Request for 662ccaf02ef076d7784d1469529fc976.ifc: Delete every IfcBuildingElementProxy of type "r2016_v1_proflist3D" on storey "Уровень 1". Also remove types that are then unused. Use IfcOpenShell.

First a look at what the model holds.

```python
import ifcopenshell
import ifcopenshell.util.element

model = ifcopenshell.open("662ccaf02ef076d7784d1469529fc976.ifc")
print(model.schema)
storey = next(s for s in model.by_type("IfcBuildingStorey") if s.Name == "Уровень 1")
proxies = [e for e in ifcopenshell.util.element.get_decomposition(storey) if e.is_a("IfcBuildingElementProxy")]
seen = {}
for e in proxies:
    element_type = ifcopenshell.util.element.get_type(e)
    name = element_type.Name if element_type not in (None, e) else None
    seen[name] = seen.get(name, 0) + 1
for name, count in sorted(seen.items(), key=str):
    print(count, "x", name)
```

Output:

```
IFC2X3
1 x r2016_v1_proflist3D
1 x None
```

```python
import ifcopenshell
import ifcopenshell.api.root
import ifcopenshell.util.element

model = ifcopenshell.open("662ccaf02ef076d7784d1469529fc976.ifc")

storey = next(s for s in model.by_type("IfcBuildingStorey") if s.Name == "Уровень 1")
proxies = [e for e in ifcopenshell.util.element.get_decomposition(storey) if e.is_a("IfcBuildingElementProxy")]
targets = [e for e in proxies if (t := ifcopenshell.util.element.get_type(e)) not in (None, e) and t.Name == "r2016_v1_proflist3D"]
types = {ifcopenshell.util.element.get_type(e) for e in targets} - {None, *targets}

for e in targets:
    ifcopenshell.api.root.remove_product(model, product=e)
print(len(targets), "removed")

unused = [t for t in types if not ifcopenshell.util.element.get_types(t)]
for t in unused:
    ifcopenshell.api.root.remove_product(model, product=t)
print(len(unused), "unused types removed")

model.write("662ccaf02ef076d7784d1469529fc976_updated.ifc")
```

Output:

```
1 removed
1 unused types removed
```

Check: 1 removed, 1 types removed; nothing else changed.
